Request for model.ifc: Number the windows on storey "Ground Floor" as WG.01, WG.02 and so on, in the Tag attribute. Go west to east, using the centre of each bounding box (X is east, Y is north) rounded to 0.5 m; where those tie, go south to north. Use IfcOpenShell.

First a look at what the model holds.

```python
import ifcopenshell
import ifcopenshell.util.element
import ifcopenshell.util.placement

model = ifcopenshell.open("model.ifc")
print(model.schema)
storey = next(s for s in model.by_type("IfcBuildingStorey") if s.Name == "Ground Floor")
windows = [e for e in ifcopenshell.util.element.get_decomposition(storey) if e.is_a("IfcWindow")]
for e in sorted(windows, key=lambda e: e.id()):
    origin = ifcopenshell.util.placement.get_local_placement(e.ObjectPlacement)[:3, 3]
    print(e.id(), e.Tag, e.Name, origin.round(2) + 0.0, sep=" | ")
```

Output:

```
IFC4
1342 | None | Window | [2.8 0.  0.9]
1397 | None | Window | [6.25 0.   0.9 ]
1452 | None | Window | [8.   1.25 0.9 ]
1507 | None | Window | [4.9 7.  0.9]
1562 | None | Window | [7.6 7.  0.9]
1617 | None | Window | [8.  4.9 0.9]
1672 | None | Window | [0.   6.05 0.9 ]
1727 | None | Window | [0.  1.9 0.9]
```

```python
import ifcopenshell
import ifcopenshell.geom
import ifcopenshell.util.element
import ifcopenshell.util.shape

model = ifcopenshell.open("model.ifc")
settings = ifcopenshell.geom.settings()
settings.set("use-world-coords", True)


def centre(element):
    shape = ifcopenshell.geom.create_shape(settings, element)
    return ifcopenshell.util.shape.get_bbox_centroid(shape.geometry)


storey = next(s for s in model.by_type("IfcBuildingStorey") if s.Name == "Ground Floor")
windows = [e for e in ifcopenshell.util.element.get_decomposition(storey) if e.is_a("IfcWindow")]

# Insertion points can sit at a corner or the storey origin, so sort by the geometry (in metres).
centres = {e: centre(e) for e in windows}
windows.sort(key=lambda e: (round(centres[e][0] / 0.5), centres[e][1]))

for i, e in enumerate(windows, start=1):
    number = f"WG.{i:02d}"
    e.Tag = number
    print(e.id(), number)

model.write("model-out.ifc")
```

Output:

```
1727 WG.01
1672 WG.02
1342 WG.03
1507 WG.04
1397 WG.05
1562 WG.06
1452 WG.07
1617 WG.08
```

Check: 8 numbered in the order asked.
